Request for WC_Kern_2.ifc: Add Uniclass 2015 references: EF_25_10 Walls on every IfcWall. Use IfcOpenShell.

First a look at what the model holds.

```python
import ifcopenshell

model = ifcopenshell.open("WC_Kern_2.ifc")
print(model.schema)
print("classifications:", [c.Name for c in model.by_type("IfcClassification")])
for ifc_class in ("IfcDoor", "IfcRoof", "IfcStair", "IfcWall", "IfcWindow"):
    print(ifc_class, len(model.by_type(ifc_class)))
```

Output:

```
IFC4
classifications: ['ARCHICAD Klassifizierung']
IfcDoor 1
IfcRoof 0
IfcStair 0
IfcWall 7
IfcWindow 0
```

```python
import ifcopenshell
import ifcopenshell.api.classification

model = ifcopenshell.open("WC_Kern_2.ifc")

system = ifcopenshell.api.classification.add_classification(model, classification="Uniclass 2015")

codes = {
    "IfcWall": ("EF_25_10", "Walls"),
}
for ifc_class, (code, name) in codes.items():
    products = model.by_type(ifc_class)
    ifcopenshell.api.classification.add_reference(
        model, products=products, classification=system, identification=code, name=name
    )
    print(code, len(products))

model.write("WC_Kern_2_v2.ifc")
```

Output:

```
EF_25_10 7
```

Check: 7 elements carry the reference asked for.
